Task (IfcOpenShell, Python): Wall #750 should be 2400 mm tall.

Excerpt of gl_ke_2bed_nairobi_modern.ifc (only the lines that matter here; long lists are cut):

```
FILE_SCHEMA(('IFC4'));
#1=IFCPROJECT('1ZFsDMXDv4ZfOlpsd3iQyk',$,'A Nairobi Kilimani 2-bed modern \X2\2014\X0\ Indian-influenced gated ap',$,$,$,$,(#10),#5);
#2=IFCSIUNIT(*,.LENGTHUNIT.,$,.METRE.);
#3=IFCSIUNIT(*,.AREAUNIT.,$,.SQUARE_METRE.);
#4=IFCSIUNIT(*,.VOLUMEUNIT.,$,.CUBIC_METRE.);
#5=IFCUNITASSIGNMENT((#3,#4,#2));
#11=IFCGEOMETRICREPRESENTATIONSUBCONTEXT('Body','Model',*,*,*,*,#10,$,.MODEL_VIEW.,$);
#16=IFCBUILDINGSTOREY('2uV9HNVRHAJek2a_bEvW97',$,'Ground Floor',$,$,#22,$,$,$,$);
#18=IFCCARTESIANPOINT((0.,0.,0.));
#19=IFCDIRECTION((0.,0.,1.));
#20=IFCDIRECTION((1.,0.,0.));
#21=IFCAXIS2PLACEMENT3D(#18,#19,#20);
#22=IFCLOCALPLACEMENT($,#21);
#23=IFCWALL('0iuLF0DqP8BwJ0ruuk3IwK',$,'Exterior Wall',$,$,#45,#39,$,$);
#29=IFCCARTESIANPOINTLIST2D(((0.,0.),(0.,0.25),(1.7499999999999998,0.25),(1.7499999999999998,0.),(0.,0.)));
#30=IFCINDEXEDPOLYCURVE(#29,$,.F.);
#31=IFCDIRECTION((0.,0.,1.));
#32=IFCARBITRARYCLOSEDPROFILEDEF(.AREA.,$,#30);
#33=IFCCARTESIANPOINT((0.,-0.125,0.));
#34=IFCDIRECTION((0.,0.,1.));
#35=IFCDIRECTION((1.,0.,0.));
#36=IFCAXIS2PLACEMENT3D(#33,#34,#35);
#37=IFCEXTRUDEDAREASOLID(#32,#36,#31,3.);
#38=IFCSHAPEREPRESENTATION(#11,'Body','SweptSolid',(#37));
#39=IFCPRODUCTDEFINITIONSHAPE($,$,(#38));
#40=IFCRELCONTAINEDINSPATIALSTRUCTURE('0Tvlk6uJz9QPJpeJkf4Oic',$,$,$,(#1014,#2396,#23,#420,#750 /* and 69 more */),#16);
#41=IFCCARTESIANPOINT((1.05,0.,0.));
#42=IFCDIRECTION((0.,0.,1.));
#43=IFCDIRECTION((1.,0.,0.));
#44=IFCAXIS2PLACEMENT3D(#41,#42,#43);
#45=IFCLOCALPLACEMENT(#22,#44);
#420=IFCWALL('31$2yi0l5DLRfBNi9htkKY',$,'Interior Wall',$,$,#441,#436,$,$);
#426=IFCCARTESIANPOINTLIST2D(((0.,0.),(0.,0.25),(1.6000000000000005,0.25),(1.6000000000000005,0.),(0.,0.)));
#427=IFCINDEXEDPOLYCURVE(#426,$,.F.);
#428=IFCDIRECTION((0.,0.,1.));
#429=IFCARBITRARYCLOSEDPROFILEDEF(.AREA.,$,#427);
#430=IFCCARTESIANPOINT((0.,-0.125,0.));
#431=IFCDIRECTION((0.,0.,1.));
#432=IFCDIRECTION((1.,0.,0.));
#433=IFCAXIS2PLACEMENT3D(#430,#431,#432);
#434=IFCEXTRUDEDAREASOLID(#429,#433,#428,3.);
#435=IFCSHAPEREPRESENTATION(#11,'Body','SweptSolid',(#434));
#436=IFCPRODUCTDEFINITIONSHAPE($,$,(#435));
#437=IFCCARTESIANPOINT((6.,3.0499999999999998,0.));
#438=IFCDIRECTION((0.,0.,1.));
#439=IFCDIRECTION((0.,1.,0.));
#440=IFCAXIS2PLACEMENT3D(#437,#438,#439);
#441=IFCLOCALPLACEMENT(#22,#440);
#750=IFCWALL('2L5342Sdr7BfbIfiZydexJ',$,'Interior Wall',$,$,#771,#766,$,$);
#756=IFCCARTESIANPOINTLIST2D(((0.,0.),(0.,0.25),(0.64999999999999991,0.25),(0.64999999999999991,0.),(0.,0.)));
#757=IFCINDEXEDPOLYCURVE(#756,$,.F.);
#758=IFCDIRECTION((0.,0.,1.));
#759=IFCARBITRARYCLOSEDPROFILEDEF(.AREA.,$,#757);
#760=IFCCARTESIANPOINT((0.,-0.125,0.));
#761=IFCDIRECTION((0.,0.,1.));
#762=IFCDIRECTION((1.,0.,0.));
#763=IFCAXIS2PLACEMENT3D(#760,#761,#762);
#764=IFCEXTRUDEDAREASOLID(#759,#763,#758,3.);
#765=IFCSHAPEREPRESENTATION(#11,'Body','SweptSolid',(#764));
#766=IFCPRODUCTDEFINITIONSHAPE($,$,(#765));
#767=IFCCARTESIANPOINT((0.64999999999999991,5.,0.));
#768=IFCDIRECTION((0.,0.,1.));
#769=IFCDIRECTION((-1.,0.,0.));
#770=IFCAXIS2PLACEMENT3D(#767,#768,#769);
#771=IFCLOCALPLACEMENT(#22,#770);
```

```python
import ifcopenshell
import ifcopenshell.geom
import ifcopenshell.util.representation
import ifcopenshell.util.shape
import ifcopenshell.util.unit

model = ifcopenshell.open("gl_ke_2bed_nairobi_modern.ifc")
unit_scale = ifcopenshell.util.unit.calculate_unit_scale(model)
settings = ifcopenshell.geom.settings()


def volume(element):
    """Net volume in cubic metres, openings subtracted."""
    shape = ifcopenshell.geom.create_shape(settings, element)
    return ifcopenshell.util.shape.get_volume(shape.geometry)


wall = model.by_guid("2L5342Sdr7BfbIfiZydexJ")
before = volume(wall)

body = ifcopenshell.util.representation.get_representation(wall, "Model", "Body")
solid = body.Items[0]
old_height = solid.Depth
solid.Depth = 2.4 / unit_scale
after = volume(wall)

print(f"height {old_height:g} -> {solid.Depth:g}, volume {before:.3f} -> {after:.3f} m3")

model.write("gl_ke_2bed_nairobi_modern_updated.ifc")
```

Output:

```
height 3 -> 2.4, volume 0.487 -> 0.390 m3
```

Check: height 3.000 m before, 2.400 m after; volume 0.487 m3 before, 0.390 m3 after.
